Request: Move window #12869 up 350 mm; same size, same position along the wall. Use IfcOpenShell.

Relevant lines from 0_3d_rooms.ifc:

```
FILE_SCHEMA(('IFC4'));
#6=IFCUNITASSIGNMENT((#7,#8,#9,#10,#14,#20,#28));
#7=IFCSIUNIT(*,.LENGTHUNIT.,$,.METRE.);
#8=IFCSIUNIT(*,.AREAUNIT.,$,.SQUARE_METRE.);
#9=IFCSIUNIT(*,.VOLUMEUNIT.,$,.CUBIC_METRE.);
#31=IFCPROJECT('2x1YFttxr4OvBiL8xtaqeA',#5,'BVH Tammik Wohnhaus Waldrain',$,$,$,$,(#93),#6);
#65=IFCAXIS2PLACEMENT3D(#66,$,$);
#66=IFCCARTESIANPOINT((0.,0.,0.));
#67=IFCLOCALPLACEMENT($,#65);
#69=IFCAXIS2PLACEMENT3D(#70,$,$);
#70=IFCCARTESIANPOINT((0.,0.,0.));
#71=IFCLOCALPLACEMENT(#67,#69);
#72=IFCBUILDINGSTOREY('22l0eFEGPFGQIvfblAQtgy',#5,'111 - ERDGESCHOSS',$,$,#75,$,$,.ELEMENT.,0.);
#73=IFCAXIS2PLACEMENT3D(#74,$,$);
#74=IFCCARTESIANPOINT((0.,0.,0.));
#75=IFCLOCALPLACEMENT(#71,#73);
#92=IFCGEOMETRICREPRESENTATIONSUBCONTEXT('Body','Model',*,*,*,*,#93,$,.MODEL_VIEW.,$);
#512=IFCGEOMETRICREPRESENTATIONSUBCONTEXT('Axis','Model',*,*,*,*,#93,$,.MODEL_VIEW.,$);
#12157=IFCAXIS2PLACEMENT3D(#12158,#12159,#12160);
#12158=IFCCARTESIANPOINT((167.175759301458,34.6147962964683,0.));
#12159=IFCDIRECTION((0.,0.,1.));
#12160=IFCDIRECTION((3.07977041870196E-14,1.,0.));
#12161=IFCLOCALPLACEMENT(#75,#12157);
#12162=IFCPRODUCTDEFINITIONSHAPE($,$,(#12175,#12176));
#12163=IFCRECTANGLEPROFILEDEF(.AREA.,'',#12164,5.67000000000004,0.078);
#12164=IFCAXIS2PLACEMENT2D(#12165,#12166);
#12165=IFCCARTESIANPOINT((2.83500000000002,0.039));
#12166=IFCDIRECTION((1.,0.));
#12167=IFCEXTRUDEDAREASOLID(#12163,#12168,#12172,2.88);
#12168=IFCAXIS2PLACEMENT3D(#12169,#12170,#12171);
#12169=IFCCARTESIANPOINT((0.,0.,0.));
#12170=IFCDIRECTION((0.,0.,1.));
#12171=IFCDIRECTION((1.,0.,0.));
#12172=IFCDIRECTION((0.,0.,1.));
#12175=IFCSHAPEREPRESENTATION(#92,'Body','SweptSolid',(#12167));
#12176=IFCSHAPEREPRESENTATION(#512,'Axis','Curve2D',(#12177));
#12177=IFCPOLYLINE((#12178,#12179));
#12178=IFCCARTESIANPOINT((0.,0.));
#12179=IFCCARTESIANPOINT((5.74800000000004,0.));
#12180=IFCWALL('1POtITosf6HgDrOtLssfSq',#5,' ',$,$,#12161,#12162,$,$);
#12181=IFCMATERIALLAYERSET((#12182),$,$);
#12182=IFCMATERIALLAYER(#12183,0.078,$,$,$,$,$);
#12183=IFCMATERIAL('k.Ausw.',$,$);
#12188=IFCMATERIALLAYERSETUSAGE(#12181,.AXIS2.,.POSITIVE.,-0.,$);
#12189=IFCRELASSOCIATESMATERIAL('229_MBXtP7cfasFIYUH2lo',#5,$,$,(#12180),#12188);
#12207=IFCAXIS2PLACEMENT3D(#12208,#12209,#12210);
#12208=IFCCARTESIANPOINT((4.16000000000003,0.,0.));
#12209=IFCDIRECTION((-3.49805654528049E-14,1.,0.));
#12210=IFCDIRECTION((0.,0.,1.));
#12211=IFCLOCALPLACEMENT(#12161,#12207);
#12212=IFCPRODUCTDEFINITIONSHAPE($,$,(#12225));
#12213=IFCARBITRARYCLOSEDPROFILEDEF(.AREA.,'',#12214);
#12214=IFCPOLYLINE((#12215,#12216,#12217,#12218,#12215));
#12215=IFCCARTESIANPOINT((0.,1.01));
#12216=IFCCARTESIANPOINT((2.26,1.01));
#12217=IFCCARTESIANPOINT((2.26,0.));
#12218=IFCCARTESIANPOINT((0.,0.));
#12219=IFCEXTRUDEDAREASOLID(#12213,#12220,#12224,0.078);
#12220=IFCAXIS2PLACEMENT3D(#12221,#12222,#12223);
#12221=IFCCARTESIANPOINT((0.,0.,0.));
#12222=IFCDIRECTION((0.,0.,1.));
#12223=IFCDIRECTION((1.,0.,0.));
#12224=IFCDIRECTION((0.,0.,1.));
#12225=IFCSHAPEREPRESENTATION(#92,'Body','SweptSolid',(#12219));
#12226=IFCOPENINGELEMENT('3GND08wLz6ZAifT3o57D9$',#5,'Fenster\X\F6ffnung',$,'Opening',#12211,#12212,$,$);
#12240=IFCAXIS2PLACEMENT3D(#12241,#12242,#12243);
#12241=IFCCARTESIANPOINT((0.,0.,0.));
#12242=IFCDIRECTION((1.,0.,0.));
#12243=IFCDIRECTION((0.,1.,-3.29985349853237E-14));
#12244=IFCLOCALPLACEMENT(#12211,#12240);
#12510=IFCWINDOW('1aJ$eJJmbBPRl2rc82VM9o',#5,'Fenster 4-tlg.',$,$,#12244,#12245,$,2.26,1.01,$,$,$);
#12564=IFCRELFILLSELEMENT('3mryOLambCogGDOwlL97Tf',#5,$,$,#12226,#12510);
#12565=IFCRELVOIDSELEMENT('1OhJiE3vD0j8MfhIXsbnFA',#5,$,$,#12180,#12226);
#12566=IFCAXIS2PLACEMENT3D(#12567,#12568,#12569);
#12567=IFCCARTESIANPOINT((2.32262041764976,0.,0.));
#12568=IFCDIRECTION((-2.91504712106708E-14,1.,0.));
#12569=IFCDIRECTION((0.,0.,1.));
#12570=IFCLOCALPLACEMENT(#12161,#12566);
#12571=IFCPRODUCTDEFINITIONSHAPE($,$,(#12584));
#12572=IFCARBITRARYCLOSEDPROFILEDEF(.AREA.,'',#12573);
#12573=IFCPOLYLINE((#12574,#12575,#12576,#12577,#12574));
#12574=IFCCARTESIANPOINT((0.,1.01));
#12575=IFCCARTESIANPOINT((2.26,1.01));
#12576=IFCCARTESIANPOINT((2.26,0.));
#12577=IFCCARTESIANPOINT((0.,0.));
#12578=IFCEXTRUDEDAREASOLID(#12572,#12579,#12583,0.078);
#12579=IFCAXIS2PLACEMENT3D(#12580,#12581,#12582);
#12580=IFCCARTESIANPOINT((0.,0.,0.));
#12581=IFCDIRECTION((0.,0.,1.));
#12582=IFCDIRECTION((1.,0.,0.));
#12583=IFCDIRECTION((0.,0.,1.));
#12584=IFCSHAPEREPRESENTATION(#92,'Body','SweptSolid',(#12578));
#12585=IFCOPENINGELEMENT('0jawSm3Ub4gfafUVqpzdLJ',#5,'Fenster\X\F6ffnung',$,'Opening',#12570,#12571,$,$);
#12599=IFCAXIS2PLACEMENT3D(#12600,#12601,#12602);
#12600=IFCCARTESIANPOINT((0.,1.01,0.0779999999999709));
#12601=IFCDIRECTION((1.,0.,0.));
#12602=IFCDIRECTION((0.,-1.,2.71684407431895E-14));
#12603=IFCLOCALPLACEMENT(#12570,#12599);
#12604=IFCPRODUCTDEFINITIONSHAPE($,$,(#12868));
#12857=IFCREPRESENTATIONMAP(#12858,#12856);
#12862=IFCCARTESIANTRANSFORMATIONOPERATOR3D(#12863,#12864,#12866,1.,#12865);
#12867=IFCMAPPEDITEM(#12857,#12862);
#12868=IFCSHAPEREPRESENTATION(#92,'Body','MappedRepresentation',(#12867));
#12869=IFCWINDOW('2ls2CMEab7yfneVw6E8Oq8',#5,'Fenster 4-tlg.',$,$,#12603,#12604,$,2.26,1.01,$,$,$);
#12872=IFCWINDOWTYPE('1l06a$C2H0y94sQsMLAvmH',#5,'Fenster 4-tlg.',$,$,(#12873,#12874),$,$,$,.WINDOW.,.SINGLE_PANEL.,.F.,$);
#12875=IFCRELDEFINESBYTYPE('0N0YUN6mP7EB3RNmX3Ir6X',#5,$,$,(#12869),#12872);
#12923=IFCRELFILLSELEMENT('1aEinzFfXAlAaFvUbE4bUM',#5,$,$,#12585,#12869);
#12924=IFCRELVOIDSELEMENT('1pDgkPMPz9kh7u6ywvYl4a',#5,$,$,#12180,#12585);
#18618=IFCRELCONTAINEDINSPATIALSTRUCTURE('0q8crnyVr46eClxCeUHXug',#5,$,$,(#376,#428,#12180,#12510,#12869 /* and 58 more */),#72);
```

```python
import numpy as np
import ifcopenshell
import ifcopenshell.api.geometry
import ifcopenshell.util.placement
import ifcopenshell.util.unit

model = ifcopenshell.open("0_3d_rooms.ifc")
unit_scale = ifcopenshell.util.unit.calculate_unit_scale(model)

window = model.by_guid("2ls2CMEab7yfneVw6E8Oq8")
opening = window.FillsVoids[0].RelatingOpeningElement
dz = 0.35

shift = np.array([0.0, 0.0, dz])
# The window is placed relative to its opening, so it follows when the opening moves.
matrix = ifcopenshell.util.placement.get_local_placement(opening.ObjectPlacement)
matrix[:3, 3] += shift
ifcopenshell.api.geometry.edit_object_placement(
    model, product=opening, matrix=matrix, is_si=False, should_transform_children=True
)

print(f"moved by {dz * unit_scale:+.3f} m")

model.write("0_3d_rooms_updated.ifc")
```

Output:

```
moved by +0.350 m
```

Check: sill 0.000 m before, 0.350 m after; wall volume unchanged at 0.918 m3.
